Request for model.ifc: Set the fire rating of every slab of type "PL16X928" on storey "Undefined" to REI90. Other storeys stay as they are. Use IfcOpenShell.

First a look at what the model holds.

```python
import ifcopenshell
import ifcopenshell.util.element

model = ifcopenshell.open("model.ifc")
print(model.schema)
storey = next(s for s in model.by_type("IfcBuildingStorey") if s.Name == "Undefined")
slabs = [e for e in ifcopenshell.util.element.get_decomposition(storey) if e.is_a("IfcSlab")]
seen = {}
for e in slabs:
    element_type = ifcopenshell.util.element.get_type(e)
    key = (element_type.Name if element_type != e and element_type else None, ifcopenshell.util.element.get_pset(e, "Pset_SlabCommon", "FireRating"))
    seen[key] = seen.get(key, 0) + 1
for (name, value), count in sorted(seen.items(), key=str):
    print(count, "x", name, "|", value)
```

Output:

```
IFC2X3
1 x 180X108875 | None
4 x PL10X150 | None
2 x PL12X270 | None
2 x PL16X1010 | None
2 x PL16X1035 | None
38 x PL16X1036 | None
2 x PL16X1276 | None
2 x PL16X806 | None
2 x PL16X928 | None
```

```python
import ifcopenshell
import ifcopenshell.api.pset
import ifcopenshell.util.element

model = ifcopenshell.open("model.ifc")

storey = next(s for s in model.by_type("IfcBuildingStorey") if s.Name == "Undefined")
slabs = [e for e in ifcopenshell.util.element.get_decomposition(storey) if e.is_a("IfcSlab")]

count = 0
for e in slabs:
    element_type = ifcopenshell.util.element.get_type(e)
    if element_type in (None, e) or element_type.Name != "PL16X928":
        continue
    # add_pset returns the element's existing set when there is one.
    pset = ifcopenshell.api.pset.add_pset(model, product=e, name="Pset_SlabCommon")
    ifcopenshell.api.pset.edit_pset(model, pset=pset, properties={"FireRating": "REI90"})
    count += 1

print(count, "slabs updated")

model.write("model_v2.ifc")
```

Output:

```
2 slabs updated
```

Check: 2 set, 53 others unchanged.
